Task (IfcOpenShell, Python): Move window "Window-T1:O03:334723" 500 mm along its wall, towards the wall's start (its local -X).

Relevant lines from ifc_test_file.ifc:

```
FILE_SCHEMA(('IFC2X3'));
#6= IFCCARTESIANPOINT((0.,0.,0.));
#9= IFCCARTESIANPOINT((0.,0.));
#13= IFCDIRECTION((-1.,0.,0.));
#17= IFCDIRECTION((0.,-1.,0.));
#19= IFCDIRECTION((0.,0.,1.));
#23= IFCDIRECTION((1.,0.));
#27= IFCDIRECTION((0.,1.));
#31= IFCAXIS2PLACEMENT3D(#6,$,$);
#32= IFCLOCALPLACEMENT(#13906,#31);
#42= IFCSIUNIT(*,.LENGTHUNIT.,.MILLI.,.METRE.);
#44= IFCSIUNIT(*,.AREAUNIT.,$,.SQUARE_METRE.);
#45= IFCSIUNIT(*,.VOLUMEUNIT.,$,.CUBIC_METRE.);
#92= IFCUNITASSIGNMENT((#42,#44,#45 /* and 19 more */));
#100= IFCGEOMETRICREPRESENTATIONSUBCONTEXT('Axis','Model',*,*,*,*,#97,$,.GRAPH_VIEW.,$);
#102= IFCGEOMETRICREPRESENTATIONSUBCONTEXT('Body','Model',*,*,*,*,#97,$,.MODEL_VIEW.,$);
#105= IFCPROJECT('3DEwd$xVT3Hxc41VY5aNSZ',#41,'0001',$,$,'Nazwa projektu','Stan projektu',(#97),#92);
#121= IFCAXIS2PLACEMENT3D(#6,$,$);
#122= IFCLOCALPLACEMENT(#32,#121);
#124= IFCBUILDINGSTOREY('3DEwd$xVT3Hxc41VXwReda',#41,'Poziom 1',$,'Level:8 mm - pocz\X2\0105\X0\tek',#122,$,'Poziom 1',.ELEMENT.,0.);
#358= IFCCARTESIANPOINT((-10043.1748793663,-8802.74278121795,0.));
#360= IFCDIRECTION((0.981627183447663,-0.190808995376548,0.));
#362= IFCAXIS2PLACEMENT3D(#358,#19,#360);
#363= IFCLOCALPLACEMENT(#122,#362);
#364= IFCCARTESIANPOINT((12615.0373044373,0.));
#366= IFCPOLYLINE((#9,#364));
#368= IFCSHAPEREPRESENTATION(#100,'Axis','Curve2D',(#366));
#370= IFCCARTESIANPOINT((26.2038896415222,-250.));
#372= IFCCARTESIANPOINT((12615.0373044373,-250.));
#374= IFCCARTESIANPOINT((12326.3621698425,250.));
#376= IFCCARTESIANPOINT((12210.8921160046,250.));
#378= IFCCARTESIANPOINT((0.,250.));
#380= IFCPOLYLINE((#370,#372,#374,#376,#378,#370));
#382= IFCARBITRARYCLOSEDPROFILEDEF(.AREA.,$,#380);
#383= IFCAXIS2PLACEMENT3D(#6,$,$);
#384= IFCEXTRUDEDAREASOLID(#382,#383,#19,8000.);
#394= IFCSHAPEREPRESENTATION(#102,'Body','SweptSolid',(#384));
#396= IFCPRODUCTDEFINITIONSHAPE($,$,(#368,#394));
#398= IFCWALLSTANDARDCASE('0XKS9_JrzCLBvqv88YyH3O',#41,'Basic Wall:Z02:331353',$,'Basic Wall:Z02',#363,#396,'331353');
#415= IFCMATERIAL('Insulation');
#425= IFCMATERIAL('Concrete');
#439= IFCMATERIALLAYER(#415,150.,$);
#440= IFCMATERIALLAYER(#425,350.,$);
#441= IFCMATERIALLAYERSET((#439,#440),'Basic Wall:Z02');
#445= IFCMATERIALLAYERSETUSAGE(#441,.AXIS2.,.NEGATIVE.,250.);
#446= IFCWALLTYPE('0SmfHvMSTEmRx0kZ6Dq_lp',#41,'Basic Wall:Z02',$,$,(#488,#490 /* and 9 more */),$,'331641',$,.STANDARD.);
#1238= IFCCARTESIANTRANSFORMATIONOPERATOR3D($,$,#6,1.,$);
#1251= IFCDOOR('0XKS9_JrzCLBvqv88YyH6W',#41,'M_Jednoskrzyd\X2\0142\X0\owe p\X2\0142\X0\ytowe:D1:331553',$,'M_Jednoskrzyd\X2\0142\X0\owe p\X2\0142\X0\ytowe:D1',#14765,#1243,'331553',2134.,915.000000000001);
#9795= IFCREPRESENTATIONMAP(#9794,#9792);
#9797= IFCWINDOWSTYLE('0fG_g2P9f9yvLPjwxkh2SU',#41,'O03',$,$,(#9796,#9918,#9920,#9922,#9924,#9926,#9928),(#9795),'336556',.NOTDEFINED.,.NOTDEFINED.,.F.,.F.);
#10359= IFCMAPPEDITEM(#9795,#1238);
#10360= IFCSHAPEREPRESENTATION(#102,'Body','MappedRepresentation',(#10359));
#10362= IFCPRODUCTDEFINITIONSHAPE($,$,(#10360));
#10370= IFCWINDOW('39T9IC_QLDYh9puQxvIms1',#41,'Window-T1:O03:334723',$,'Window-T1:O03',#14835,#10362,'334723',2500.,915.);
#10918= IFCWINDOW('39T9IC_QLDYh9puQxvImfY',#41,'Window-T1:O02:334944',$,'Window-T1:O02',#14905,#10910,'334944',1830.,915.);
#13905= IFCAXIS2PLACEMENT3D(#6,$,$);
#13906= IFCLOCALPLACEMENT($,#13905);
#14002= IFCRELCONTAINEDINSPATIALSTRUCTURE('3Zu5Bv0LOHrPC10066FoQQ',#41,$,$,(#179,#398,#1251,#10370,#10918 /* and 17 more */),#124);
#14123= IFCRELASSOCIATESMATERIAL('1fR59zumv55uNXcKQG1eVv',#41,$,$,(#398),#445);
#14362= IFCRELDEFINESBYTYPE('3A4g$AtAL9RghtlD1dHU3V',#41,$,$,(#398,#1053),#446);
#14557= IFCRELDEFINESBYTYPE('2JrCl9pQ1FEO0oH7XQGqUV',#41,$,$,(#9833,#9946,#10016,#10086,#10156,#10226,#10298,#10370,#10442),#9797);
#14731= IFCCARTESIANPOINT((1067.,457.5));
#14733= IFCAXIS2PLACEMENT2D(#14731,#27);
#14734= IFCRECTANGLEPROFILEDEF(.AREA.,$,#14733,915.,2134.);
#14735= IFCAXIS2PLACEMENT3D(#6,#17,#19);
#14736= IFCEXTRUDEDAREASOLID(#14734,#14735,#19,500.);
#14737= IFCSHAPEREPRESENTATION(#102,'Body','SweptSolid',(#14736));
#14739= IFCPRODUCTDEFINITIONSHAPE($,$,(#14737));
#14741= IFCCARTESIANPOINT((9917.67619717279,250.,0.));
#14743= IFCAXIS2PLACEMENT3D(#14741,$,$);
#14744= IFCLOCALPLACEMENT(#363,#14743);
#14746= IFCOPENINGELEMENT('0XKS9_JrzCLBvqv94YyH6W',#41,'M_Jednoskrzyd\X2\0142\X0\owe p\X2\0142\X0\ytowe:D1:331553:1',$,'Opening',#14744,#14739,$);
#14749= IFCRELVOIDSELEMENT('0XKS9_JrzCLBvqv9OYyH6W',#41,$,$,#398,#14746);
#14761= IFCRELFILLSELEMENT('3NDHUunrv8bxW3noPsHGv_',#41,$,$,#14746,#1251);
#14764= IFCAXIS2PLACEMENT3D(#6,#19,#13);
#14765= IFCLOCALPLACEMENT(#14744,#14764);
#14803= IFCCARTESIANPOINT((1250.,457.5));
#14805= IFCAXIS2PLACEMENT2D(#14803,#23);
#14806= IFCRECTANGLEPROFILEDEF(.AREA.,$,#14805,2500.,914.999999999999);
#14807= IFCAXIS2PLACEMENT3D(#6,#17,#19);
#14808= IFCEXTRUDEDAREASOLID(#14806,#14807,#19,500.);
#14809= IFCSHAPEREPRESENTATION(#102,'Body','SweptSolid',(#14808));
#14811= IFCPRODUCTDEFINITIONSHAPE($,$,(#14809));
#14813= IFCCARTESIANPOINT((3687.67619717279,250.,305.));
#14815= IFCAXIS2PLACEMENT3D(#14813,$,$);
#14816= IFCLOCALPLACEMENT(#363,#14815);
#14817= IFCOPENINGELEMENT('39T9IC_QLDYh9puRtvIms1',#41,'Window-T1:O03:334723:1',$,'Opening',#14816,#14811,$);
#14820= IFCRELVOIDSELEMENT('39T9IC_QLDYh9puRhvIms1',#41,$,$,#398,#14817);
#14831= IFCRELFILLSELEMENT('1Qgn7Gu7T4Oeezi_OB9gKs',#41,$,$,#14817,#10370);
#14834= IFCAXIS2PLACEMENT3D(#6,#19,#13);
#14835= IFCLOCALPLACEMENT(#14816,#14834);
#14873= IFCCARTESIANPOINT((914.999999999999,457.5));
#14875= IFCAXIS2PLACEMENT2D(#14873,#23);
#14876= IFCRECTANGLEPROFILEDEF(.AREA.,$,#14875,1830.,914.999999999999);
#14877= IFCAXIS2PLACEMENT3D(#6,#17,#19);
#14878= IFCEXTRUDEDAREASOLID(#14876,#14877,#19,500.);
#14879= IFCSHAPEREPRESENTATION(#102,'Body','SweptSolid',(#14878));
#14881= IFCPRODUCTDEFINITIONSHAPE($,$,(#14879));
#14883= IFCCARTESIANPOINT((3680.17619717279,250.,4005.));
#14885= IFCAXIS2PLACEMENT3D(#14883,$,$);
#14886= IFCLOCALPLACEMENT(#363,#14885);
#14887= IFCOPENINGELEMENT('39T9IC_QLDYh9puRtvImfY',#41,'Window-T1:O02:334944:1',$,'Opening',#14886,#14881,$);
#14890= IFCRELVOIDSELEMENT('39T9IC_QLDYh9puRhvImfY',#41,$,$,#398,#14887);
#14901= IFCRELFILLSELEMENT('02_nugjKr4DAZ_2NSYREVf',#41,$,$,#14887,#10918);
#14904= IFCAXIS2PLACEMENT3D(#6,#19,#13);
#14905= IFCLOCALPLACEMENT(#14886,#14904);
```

```python
import ifcopenshell
import ifcopenshell.api.geometry
import ifcopenshell.util.placement
import ifcopenshell.util.unit

model = ifcopenshell.open("ifc_test_file.ifc")
unit_scale = ifcopenshell.util.unit.calculate_unit_scale(model)

window = model.by_id(10370)
opening = window.FillsVoids[0].RelatingOpeningElement
wall = opening.VoidsElements[0].RelatingBuildingElement

wall_matrix = ifcopenshell.util.placement.get_local_placement(wall.ObjectPlacement)
shift = wall_matrix[:3, 0] * -0.5 / unit_scale
before = ifcopenshell.util.placement.get_local_placement(window.ObjectPlacement)[:3, 3].copy()

# The window is placed relative to its opening, so it follows when the opening moves.
matrix = ifcopenshell.util.placement.get_local_placement(opening.ObjectPlacement)
matrix[:3, 3] += shift
ifcopenshell.api.geometry.edit_object_placement(
    model, product=opening, matrix=matrix, is_si=False, should_transform_children=True
)

after = ifcopenshell.util.placement.get_local_placement(window.ObjectPlacement)[:3, 3]
print("window moved by", (after - before).round(3) + 0.0)

model.write("ifc_test_file-out.ifc")
```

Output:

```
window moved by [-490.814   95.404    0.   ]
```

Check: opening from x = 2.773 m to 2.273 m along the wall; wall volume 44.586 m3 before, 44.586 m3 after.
